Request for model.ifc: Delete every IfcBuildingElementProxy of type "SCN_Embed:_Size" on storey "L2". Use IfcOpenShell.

First a look at what the model holds.

```python
import ifcopenshell
import ifcopenshell.util.element

model = ifcopenshell.open("model.ifc")
print(model.schema)
storey = next(s for s in model.by_type("IfcBuildingStorey") if s.Name == "L2")
proxies = [e for e in ifcopenshell.util.element.get_decomposition(storey) if e.is_a("IfcBuildingElementProxy")]
seen = {}
for e in proxies:
    element_type = ifcopenshell.util.element.get_type(e)
    name = element_type.Name if element_type not in (None, e) else None
    seen[name] = seen.get(name, 0) + 1
for name, count in sorted(seen.items(), key=str):
    print(count, "x", name)
```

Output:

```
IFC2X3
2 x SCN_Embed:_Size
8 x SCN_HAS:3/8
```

```python
import ifcopenshell
import ifcopenshell.api.root
import ifcopenshell.util.element

model = ifcopenshell.open("model.ifc")

storey = next(s for s in model.by_type("IfcBuildingStorey") if s.Name == "L2")
proxies = [e for e in ifcopenshell.util.element.get_decomposition(storey) if e.is_a("IfcBuildingElementProxy")]
targets = [e for e in proxies if (t := ifcopenshell.util.element.get_type(e)) not in (None, e) and t.Name == "SCN_Embed:_Size"]

for e in targets:
    ifcopenshell.api.root.remove_product(model, product=e)
print(len(targets), "removed")

model.write("model_rev.ifc")
```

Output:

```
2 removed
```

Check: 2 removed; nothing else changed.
